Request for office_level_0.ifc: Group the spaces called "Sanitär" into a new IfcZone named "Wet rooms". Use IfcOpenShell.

First a look at what the model holds.

```python
import ifcopenshell

model = ifcopenshell.open("office_level_0.ifc")
print(model.schema)
seen = {}
for space in model.by_type("IfcSpace"):
    seen[space.LongName] = seen.get(space.LongName, 0) + 1
for name, count in sorted(seen.items(), key=str):
    print(count, "x", name)
print("zones:", [z.Name for z in model.by_type("IfcZone")][:20])
```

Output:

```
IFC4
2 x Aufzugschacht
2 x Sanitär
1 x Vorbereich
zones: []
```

```python
import ifcopenshell
import ifcopenshell.api.group
import ifcopenshell.api.root

model = ifcopenshell.open("office_level_0.ifc")

names = {"Sanitär"}
spaces = [s for s in model.by_type("IfcSpace") if s.LongName in names]

zone = ifcopenshell.api.root.create_entity(model, ifc_class="IfcZone", name="Wet rooms")
ifcopenshell.api.group.assign_group(model, products=spaces, group=zone)
print(len(spaces), "spaces in", zone.Name)

model.write("office_level_0_v2.ifc")
```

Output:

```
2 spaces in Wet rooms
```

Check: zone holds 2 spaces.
